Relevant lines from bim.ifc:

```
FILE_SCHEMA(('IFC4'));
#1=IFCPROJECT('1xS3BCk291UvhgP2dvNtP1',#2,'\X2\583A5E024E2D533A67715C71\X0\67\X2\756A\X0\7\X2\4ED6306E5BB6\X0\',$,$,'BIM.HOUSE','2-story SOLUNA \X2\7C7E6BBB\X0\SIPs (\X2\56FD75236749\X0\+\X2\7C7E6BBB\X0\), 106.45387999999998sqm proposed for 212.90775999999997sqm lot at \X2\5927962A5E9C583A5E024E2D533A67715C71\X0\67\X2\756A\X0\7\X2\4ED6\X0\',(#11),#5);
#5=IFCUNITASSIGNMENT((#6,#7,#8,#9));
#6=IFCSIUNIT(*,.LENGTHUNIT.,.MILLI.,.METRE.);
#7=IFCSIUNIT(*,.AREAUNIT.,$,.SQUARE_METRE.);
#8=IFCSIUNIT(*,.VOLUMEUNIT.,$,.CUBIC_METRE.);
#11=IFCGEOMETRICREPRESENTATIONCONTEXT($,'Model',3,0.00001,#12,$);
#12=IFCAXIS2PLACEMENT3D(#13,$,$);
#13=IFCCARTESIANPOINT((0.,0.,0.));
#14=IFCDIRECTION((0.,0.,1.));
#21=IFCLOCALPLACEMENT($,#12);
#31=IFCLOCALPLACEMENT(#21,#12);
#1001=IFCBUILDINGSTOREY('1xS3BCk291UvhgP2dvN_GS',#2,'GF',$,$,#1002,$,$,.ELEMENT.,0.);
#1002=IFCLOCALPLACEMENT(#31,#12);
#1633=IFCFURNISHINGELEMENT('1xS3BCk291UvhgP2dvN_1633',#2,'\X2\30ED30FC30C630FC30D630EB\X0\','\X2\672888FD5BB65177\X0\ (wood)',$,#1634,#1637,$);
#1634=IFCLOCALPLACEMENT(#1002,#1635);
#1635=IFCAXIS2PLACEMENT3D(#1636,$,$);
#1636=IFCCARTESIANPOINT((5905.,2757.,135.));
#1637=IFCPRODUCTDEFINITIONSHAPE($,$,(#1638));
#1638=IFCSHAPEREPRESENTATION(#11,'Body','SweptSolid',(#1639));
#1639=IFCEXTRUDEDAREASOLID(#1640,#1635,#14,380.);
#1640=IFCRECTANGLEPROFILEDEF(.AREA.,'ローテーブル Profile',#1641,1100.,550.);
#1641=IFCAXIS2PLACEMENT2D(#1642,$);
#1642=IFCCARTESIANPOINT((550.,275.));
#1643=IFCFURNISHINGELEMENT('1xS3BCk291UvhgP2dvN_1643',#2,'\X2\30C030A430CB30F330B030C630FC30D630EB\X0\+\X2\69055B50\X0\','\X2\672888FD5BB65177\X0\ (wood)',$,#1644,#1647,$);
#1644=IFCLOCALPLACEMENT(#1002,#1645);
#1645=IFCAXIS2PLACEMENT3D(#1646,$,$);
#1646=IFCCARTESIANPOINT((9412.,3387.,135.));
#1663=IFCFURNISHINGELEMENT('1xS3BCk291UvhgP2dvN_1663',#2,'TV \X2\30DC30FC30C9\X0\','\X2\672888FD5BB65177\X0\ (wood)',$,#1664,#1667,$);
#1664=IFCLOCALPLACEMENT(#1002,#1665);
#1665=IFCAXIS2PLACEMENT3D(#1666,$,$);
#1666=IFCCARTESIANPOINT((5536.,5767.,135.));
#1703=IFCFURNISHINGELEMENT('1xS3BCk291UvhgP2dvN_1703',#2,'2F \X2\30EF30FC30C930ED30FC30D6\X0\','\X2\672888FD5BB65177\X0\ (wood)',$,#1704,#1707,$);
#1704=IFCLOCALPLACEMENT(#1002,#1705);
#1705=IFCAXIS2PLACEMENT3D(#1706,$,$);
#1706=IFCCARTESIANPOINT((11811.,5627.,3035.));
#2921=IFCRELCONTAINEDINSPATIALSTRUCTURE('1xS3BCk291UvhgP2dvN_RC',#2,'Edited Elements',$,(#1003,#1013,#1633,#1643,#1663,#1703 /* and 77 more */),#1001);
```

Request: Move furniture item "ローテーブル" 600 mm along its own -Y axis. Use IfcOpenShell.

```python
import ifcopenshell
import ifcopenshell.api.geometry
import ifcopenshell.util.placement

model = ifcopenshell.open("bim.ifc")

item = model.by_id(1633)
matrix = ifcopenshell.util.placement.get_local_placement(item.ObjectPlacement)
matrix[:3, 3] -= matrix[:3, 1] * 600.0
ifcopenshell.api.geometry.edit_object_placement(model, product=item, matrix=matrix, is_si=False)

print(ifcopenshell.util.placement.get_local_placement(item.ObjectPlacement).round(3) + 0.0)

model.write("bim-out.ifc")
```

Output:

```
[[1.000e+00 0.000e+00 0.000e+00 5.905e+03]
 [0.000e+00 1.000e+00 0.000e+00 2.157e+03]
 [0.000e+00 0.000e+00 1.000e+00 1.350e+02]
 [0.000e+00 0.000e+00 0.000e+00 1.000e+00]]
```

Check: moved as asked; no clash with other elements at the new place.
